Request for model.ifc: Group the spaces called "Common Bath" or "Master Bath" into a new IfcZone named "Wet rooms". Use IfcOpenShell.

First a look at what the model holds.

```python
import ifcopenshell

model = ifcopenshell.open("model.ifc")
print(model.schema)
seen = {}
for space in model.by_type("IfcSpace"):
    seen[space.LongName] = seen.get(space.LongName, 0) + 1
for name, count in sorted(seen.items(), key=str):
    print(count, "x", name)
print("zones:", [z.Name for z in model.by_type("IfcZone")][:20])
```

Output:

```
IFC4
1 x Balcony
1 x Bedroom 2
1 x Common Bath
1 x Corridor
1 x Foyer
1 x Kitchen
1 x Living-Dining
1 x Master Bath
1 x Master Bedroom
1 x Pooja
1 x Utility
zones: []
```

```python
import ifcopenshell
import ifcopenshell.api.group
import ifcopenshell.api.root

model = ifcopenshell.open("model.ifc")

names = {"Common Bath", "Master Bath"}
spaces = [s for s in model.by_type("IfcSpace") if s.LongName in names]

zone = ifcopenshell.api.root.create_entity(model, ifc_class="IfcZone", name="Wet rooms")
ifcopenshell.api.group.assign_group(model, products=spaces, group=zone)
print(len(spaces), "spaces in", zone.Name)

model.write("model_updated.ifc")
```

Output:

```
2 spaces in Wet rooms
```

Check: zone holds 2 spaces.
